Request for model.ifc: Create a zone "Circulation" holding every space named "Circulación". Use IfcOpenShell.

First a look at what the model holds.

```python
import ifcopenshell

model = ifcopenshell.open("model.ifc")
print(model.schema)
seen = {}
for space in model.by_type("IfcSpace"):
    seen[space.LongName] = seen.get(space.LongName, 0) + 1
for name, count in sorted(seen.items(), key=str):
    print(count, "x", name)
print("zones:", [z.Name for z in model.by_type("IfcZone")][:20])
```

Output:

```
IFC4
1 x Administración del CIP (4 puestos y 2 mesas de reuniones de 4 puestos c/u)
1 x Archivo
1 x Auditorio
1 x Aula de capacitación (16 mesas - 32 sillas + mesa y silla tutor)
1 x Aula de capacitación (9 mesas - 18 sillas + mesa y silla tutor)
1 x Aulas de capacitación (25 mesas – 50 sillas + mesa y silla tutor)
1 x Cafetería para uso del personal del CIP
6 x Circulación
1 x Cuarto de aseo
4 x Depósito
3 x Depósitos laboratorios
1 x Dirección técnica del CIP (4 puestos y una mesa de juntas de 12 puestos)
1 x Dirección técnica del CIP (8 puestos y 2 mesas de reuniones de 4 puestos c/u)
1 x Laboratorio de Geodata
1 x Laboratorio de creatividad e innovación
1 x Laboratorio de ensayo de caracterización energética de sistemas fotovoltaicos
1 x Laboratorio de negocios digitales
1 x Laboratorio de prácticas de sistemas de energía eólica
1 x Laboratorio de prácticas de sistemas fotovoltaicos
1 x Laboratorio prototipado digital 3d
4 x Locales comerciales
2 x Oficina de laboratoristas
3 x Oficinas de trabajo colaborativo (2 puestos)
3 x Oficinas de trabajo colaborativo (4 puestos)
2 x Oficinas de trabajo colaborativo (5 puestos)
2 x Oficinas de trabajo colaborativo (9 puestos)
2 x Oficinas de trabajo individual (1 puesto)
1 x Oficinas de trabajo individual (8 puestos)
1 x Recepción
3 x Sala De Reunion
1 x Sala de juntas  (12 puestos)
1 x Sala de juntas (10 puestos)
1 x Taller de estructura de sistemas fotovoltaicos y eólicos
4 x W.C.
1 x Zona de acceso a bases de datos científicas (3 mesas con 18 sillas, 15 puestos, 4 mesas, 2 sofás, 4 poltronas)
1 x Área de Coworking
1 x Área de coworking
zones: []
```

```python
import ifcopenshell
import ifcopenshell.api.group
import ifcopenshell.api.root

model = ifcopenshell.open("model.ifc")

names = {"Circulación"}
spaces = [s for s in model.by_type("IfcSpace") if s.LongName in names]

zone = ifcopenshell.api.root.create_entity(model, ifc_class="IfcZone", name="Circulation")
ifcopenshell.api.group.assign_group(model, products=spaces, group=zone)
print(len(spaces), "spaces in", zone.Name)

model.write("model_edited.ifc")
```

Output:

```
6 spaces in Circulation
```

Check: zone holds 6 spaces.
